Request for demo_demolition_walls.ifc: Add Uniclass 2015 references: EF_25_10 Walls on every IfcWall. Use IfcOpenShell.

First a look at what the model holds.

```python
import ifcopenshell

model = ifcopenshell.open("demo_demolition_walls.ifc")
print(model.schema)
print("classifications:", [c.Name for c in model.by_type("IfcClassification")])
for ifc_class in ("IfcDoor", "IfcRoof", "IfcStair", "IfcWall", "IfcWindow"):
    print(ifc_class, len(model.by_type(ifc_class)))
```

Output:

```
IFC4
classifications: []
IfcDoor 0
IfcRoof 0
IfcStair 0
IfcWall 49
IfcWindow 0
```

```python
import ifcopenshell
import ifcopenshell.api.classification

model = ifcopenshell.open("demo_demolition_walls.ifc")

system = ifcopenshell.api.classification.add_classification(model, classification="Uniclass 2015")

codes = {
    "IfcWall": ("EF_25_10", "Walls"),
}
for ifc_class, (code, name) in codes.items():
    products = model.by_type(ifc_class)
    ifcopenshell.api.classification.add_reference(
        model, products=products, classification=system, identification=code, name=name
    )
    print(code, len(products))

model.write("demo_demolition_walls_v2.ifc")
```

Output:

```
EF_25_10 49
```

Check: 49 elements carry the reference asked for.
